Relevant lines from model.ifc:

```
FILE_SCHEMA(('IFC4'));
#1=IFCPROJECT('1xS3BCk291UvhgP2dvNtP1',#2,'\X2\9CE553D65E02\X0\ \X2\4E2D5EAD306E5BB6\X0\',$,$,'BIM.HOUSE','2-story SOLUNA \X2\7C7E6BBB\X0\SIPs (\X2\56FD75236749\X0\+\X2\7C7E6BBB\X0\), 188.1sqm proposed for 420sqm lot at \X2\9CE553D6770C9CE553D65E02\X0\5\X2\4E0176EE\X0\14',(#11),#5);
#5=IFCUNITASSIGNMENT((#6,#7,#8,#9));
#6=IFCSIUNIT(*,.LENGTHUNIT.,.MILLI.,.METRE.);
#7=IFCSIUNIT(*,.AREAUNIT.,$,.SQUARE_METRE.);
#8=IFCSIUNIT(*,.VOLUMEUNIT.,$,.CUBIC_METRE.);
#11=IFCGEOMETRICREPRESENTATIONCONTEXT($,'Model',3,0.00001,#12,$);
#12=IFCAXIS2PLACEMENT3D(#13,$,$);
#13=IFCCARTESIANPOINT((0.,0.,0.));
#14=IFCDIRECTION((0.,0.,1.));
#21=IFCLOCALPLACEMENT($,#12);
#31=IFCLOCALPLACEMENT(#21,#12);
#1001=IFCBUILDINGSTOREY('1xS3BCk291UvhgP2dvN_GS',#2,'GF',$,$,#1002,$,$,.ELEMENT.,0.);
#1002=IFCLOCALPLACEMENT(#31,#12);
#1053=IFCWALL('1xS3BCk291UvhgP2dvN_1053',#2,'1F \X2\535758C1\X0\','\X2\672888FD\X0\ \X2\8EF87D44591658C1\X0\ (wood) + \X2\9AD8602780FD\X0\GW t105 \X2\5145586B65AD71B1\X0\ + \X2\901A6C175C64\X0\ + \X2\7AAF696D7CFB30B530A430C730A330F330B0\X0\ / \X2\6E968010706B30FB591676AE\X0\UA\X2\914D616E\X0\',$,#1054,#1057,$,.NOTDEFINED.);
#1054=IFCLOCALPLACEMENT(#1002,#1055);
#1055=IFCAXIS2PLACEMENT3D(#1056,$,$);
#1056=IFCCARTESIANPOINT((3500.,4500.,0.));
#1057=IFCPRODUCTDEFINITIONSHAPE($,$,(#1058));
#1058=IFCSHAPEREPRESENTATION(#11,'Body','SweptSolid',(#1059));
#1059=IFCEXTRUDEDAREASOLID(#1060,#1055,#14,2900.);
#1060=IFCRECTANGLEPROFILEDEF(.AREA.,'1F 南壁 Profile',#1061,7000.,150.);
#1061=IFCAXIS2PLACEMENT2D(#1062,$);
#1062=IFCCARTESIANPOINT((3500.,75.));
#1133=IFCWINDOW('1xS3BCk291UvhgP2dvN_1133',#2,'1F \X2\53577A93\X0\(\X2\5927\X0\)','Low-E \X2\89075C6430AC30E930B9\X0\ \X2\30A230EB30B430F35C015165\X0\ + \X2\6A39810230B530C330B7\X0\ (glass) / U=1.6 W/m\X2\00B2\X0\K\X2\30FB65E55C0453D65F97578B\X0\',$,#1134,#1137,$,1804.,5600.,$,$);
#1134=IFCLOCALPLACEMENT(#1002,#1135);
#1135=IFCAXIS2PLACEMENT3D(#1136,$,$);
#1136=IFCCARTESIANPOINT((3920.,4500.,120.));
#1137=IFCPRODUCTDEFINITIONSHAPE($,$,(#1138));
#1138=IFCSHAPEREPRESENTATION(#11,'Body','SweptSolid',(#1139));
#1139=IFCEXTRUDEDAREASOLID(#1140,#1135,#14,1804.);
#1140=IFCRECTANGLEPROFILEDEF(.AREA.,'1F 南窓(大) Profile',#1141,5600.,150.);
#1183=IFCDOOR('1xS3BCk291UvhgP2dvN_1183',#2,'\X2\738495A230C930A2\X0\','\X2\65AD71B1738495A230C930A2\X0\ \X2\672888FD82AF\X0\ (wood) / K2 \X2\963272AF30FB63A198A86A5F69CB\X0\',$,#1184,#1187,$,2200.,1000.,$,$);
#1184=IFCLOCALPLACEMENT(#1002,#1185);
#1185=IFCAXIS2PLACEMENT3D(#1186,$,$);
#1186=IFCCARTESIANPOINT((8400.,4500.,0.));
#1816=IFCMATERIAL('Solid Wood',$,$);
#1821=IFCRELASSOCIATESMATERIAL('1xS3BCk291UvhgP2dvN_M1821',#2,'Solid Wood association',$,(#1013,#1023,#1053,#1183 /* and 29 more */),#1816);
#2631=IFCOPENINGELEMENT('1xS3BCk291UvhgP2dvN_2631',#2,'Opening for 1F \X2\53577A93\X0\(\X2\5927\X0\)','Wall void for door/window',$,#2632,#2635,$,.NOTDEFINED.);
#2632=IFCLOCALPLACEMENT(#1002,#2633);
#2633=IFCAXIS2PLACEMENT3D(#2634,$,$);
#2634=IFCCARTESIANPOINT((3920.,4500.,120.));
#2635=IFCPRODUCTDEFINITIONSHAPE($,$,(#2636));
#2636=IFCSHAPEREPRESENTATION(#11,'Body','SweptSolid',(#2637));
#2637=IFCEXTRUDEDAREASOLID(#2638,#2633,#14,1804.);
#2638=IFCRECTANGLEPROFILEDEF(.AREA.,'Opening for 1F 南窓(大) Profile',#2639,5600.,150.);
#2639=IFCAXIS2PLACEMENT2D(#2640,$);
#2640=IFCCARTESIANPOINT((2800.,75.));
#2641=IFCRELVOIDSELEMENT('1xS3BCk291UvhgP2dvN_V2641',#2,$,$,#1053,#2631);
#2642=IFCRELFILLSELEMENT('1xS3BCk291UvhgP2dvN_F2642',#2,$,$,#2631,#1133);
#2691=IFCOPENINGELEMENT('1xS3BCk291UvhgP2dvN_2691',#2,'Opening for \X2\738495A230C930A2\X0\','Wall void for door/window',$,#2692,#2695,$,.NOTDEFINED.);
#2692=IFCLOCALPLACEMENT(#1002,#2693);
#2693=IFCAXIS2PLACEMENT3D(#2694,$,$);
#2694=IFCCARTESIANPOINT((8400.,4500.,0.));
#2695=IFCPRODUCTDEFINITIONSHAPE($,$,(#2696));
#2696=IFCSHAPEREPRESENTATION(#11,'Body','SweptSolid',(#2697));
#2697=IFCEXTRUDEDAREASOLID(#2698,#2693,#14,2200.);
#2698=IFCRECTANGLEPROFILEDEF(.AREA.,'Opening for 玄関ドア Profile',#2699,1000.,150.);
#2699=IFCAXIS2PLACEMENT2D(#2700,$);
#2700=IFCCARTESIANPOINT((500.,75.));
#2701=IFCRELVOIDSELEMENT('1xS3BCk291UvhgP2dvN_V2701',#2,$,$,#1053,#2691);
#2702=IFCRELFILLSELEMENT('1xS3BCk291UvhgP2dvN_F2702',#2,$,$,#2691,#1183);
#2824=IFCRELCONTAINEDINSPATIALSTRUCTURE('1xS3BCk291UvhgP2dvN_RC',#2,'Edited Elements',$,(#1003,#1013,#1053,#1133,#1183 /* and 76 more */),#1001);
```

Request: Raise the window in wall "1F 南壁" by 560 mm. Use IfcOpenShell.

```python
import numpy as np
import ifcopenshell
import ifcopenshell.api.geometry
import ifcopenshell.util.placement
import ifcopenshell.util.unit

model = ifcopenshell.open("model.ifc")
unit_scale = ifcopenshell.util.unit.calculate_unit_scale(model)

window = model.by_id(1133)
opening = window.FillsVoids[0].RelatingOpeningElement
dz = 0.56 / unit_scale

shift = np.array([0.0, 0.0, dz])
# The window is not placed relative to its opening, so move both.
for product in (opening, window):
    matrix = ifcopenshell.util.placement.get_local_placement(product.ObjectPlacement)
    matrix[:3, 3] += shift
    ifcopenshell.api.geometry.edit_object_placement(model, product=product, matrix=matrix, is_si=False)

print(f"moved by {dz * unit_scale:+.3f} m")

model.write("model-out.ifc")
```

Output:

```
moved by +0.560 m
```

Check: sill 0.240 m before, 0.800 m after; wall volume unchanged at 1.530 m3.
